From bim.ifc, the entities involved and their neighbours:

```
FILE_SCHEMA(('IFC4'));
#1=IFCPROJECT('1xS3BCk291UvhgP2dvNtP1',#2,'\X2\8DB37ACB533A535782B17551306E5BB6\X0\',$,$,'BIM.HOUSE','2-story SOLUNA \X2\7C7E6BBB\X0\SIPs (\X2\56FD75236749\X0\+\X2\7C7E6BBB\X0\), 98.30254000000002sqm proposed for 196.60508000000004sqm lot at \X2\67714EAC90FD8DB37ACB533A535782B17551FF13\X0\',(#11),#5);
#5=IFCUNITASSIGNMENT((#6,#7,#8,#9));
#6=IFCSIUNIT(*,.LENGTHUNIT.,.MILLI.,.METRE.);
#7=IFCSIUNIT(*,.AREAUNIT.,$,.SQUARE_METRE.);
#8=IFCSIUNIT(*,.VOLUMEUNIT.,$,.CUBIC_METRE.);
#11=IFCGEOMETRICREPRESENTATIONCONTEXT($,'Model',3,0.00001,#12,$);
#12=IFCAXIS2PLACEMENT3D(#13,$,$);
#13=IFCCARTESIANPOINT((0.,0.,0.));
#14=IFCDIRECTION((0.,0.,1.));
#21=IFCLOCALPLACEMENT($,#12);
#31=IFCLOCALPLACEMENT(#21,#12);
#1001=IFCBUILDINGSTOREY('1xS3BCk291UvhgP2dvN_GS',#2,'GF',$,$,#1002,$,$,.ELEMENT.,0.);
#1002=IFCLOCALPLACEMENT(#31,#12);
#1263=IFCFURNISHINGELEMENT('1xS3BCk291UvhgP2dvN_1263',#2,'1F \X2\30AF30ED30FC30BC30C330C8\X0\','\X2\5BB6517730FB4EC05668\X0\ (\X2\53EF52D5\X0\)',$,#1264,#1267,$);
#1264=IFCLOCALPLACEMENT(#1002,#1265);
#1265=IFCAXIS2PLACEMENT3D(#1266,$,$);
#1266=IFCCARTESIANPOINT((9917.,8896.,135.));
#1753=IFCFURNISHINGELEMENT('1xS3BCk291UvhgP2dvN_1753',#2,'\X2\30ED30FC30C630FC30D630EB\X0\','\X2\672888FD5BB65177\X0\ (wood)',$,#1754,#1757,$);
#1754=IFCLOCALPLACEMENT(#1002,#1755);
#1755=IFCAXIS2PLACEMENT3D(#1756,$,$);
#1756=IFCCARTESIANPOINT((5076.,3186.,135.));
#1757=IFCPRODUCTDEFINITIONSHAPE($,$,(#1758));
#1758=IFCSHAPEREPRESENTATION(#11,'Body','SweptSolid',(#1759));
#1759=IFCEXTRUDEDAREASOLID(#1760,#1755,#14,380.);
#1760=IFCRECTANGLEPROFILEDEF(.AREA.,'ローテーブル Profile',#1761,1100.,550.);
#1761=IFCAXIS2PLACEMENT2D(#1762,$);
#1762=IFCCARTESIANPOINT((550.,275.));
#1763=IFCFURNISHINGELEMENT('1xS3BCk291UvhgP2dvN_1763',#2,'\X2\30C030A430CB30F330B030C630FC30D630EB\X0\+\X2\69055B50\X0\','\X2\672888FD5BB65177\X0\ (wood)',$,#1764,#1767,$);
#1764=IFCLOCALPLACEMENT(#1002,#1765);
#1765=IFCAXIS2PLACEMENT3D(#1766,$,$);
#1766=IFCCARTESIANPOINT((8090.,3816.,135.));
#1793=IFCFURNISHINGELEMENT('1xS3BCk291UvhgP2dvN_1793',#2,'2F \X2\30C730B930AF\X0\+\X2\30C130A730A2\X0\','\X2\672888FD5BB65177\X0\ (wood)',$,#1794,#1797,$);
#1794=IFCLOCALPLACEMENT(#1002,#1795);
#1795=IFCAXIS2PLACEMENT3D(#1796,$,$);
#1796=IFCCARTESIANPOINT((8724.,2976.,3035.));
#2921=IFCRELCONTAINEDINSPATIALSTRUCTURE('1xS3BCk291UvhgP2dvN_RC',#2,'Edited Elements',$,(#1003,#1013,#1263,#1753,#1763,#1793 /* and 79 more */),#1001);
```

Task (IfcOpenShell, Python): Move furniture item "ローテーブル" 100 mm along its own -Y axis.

```python
import ifcopenshell
import ifcopenshell.api.geometry
import ifcopenshell.util.placement
import ifcopenshell.util.unit

model = ifcopenshell.open("bim.ifc")
unit_scale = ifcopenshell.util.unit.calculate_unit_scale(model)

item = model.by_id(1753)
matrix = ifcopenshell.util.placement.get_local_placement(item.ObjectPlacement)
matrix[:3, 3] -= matrix[:3, 1] * 0.1 / unit_scale
ifcopenshell.api.geometry.edit_object_placement(model, product=item, matrix=matrix, is_si=False)

print(ifcopenshell.util.placement.get_local_placement(item.ObjectPlacement).round(3) + 0.0)

model.write("bim_edited.ifc")
```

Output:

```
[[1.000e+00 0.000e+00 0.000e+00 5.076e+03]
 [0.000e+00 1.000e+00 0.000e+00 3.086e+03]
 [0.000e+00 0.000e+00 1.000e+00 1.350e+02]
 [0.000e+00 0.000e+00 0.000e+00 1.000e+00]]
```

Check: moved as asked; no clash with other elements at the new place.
